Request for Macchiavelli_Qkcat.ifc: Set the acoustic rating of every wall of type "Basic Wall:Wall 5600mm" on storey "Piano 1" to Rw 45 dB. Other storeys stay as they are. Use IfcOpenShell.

First a look at what the model holds.

```python
import ifcopenshell
import ifcopenshell.util.element

model = ifcopenshell.open("Macchiavelli_Qkcat.ifc")
print(model.schema)
storey = next(s for s in model.by_type("IfcBuildingStorey") if s.Name == "Piano 1")
walls = [e for e in ifcopenshell.util.element.get_decomposition(storey) if e.is_a("IfcWall")]
seen = {}
for e in walls:
    element_type = ifcopenshell.util.element.get_type(e)
    key = (element_type.Name if element_type != e and element_type else None, ifcopenshell.util.element.get_pset(e, "Pset_WallCommon", "AcousticRating"))
    seen[key] = seen.get(key, 0) + 1
for (name, value), count in sorted(seen.items(), key=str):
    print(count, "x", name, "|", value)
```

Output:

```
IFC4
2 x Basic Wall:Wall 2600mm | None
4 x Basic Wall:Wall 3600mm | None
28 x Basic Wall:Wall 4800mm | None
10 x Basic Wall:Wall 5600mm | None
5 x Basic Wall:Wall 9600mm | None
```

```python
import ifcopenshell
import ifcopenshell.api.pset
import ifcopenshell.util.element

model = ifcopenshell.open("Macchiavelli_Qkcat.ifc")

storey = next(s for s in model.by_type("IfcBuildingStorey") if s.Name == "Piano 1")
walls = [e for e in ifcopenshell.util.element.get_decomposition(storey) if e.is_a("IfcWall")]

count = 0
for e in walls:
    element_type = ifcopenshell.util.element.get_type(e)
    if element_type in (None, e) or element_type.Name != "Basic Wall:Wall 5600mm":
        continue
    # add_pset returns the element's existing set when there is one.
    pset = ifcopenshell.api.pset.add_pset(model, product=e, name="Pset_WallCommon")
    ifcopenshell.api.pset.edit_pset(model, pset=pset, properties={"AcousticRating": "Rw 45 dB"})
    count += 1

print(count, "walls updated")

model.write("Macchiavelli_Qkcat-out.ifc")
```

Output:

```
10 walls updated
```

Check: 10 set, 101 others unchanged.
